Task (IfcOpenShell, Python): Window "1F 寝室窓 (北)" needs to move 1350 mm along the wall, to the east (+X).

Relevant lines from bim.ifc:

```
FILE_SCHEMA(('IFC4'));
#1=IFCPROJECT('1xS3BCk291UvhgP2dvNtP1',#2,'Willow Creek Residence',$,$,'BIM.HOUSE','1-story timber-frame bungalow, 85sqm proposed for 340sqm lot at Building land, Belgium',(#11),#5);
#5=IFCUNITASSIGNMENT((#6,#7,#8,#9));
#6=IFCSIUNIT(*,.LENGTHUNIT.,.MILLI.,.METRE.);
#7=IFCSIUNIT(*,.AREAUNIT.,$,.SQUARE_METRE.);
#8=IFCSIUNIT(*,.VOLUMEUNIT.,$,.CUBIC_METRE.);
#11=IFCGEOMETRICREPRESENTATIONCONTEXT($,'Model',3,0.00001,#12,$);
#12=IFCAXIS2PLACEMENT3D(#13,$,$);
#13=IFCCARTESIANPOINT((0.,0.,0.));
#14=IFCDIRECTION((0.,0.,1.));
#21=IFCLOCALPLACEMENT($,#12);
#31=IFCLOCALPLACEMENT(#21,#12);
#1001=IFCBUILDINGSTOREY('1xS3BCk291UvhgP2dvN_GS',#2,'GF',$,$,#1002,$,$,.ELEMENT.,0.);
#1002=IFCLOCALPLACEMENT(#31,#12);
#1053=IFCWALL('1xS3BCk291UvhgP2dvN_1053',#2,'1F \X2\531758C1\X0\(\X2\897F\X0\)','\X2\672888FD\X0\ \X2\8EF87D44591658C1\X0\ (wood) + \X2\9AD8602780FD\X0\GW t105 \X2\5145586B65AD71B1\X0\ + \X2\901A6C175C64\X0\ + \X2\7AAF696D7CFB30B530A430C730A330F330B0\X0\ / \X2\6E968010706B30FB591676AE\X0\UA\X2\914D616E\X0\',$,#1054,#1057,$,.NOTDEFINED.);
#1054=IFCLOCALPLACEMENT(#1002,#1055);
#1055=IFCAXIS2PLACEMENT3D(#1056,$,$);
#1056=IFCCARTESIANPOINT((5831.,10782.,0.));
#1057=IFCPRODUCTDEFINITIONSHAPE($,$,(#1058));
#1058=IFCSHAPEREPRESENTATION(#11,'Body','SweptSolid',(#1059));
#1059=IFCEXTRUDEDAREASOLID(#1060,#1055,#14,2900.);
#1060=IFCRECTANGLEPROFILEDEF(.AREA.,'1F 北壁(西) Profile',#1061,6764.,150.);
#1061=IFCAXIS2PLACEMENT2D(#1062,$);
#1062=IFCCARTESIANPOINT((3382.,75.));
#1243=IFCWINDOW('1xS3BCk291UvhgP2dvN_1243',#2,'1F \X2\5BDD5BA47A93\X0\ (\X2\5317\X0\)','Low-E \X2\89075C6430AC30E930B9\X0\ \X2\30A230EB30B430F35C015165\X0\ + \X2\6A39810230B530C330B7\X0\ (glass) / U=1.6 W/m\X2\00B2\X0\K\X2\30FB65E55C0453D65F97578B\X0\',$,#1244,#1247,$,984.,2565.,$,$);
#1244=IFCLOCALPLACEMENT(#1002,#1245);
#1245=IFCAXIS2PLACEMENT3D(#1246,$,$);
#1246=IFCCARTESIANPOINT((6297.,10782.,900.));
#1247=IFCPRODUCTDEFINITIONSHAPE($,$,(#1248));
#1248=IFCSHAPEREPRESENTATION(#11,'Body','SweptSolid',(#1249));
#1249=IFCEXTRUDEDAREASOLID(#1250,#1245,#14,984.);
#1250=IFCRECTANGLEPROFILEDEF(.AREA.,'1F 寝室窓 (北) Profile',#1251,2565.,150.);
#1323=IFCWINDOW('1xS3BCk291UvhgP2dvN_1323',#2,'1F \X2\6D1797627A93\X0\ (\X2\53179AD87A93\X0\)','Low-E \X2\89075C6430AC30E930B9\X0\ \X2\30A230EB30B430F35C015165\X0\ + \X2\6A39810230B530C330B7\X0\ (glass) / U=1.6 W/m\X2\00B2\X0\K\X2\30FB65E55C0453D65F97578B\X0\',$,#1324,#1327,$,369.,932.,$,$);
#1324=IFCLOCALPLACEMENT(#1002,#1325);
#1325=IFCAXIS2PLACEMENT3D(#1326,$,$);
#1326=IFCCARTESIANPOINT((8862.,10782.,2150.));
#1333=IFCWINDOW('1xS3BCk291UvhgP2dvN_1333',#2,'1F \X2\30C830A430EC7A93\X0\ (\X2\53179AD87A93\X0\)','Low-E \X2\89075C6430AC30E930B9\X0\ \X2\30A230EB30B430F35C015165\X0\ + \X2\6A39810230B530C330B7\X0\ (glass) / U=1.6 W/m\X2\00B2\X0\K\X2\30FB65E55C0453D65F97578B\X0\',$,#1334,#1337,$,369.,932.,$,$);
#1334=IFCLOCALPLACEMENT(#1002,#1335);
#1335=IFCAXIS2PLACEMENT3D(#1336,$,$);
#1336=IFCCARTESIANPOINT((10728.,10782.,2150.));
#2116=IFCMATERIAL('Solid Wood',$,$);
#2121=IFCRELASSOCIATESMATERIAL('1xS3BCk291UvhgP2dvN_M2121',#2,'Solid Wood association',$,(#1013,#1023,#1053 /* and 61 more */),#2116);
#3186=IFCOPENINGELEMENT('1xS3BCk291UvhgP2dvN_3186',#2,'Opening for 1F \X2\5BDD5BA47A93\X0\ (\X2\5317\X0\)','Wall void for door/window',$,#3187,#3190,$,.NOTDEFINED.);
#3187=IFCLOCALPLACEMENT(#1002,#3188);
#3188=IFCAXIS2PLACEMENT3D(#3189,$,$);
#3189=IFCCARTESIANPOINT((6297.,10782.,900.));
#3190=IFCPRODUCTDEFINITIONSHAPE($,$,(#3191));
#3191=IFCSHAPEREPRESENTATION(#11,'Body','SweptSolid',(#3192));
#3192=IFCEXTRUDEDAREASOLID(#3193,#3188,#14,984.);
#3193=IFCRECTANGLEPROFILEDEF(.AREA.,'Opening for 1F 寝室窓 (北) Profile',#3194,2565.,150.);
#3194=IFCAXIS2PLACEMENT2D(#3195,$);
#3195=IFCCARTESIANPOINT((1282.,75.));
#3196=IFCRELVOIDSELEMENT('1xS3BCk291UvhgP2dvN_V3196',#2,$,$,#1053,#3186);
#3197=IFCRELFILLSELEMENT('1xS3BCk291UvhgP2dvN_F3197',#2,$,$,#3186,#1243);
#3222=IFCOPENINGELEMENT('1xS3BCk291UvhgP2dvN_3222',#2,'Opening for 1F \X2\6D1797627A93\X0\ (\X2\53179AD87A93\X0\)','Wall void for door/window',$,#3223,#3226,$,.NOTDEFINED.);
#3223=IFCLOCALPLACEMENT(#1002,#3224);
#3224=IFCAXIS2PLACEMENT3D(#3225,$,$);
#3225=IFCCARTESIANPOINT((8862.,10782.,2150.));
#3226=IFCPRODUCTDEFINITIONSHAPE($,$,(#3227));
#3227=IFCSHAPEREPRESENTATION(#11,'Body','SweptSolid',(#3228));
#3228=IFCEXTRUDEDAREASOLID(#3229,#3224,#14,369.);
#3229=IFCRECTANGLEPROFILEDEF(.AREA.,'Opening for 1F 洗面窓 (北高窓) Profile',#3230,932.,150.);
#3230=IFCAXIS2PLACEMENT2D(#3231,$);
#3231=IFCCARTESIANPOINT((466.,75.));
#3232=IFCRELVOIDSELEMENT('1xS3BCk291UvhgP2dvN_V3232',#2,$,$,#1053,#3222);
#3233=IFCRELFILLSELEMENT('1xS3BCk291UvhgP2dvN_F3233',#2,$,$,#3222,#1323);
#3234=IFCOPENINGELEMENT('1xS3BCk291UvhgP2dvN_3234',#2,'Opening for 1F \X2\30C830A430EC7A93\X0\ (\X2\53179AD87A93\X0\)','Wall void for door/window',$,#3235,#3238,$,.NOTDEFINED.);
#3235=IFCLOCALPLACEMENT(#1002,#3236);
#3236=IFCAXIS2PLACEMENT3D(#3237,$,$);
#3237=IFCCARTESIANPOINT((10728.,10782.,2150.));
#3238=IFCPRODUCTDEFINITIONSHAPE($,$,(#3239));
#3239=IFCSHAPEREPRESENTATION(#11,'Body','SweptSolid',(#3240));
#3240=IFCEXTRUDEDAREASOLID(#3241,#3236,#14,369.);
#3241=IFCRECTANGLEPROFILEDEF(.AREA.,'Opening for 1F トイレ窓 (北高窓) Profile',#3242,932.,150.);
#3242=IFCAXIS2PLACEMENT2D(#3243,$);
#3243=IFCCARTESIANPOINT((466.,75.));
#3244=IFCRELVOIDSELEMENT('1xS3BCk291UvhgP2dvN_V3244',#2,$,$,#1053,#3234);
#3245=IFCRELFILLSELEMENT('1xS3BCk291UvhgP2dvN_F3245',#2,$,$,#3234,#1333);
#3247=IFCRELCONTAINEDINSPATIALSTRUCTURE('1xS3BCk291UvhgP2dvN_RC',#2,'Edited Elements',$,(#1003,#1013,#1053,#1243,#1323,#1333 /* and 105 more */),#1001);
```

```python
import ifcopenshell
import ifcopenshell.api.geometry
import ifcopenshell.util.placement

model = ifcopenshell.open("bim.ifc")

window = model.by_guid("1xS3BCk291UvhgP2dvN_1243")
opening = window.FillsVoids[0].RelatingOpeningElement
wall = opening.VoidsElements[0].RelatingBuildingElement

wall_matrix = ifcopenshell.util.placement.get_local_placement(wall.ObjectPlacement)
shift = wall_matrix[:3, 0] * 1350.0
before = ifcopenshell.util.placement.get_local_placement(window.ObjectPlacement)[:3, 3].copy()

# The window is not placed relative to its opening, so move both.
for product in (opening, window):
    matrix = ifcopenshell.util.placement.get_local_placement(product.ObjectPlacement)
    matrix[:3, 3] += shift
    ifcopenshell.api.geometry.edit_object_placement(model, product=product, matrix=matrix, is_si=False)

after = ifcopenshell.util.placement.get_local_placement(window.ObjectPlacement)[:3, 3]
print("window moved by", (after - before).round(3) + 0.0)

model.write("bim_rev.ifc")
```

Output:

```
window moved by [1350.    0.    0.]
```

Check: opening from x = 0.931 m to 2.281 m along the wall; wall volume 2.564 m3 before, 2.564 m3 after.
